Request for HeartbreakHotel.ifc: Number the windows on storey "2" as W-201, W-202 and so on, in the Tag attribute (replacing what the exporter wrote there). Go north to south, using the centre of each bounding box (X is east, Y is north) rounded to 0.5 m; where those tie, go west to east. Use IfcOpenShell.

First a look at what the model holds.

```python
import ifcopenshell
import ifcopenshell.util.element
import ifcopenshell.util.placement

model = ifcopenshell.open("HeartbreakHotel.ifc")
print(model.schema)
storey = next(s for s in model.by_type("IfcBuildingStorey") if s.Name == "2")
windows = [e for e in ifcopenshell.util.element.get_decomposition(storey) if e.is_a("IfcWindow")]
for e in sorted(windows, key=lambda e: e.id()):
    origin = ifcopenshell.util.placement.get_local_placement(e.ObjectPlacement)[:3, 3]
    print(e.id(), e.Tag, e.Name, origin.round(2) + 0.0, sep=" | ")
```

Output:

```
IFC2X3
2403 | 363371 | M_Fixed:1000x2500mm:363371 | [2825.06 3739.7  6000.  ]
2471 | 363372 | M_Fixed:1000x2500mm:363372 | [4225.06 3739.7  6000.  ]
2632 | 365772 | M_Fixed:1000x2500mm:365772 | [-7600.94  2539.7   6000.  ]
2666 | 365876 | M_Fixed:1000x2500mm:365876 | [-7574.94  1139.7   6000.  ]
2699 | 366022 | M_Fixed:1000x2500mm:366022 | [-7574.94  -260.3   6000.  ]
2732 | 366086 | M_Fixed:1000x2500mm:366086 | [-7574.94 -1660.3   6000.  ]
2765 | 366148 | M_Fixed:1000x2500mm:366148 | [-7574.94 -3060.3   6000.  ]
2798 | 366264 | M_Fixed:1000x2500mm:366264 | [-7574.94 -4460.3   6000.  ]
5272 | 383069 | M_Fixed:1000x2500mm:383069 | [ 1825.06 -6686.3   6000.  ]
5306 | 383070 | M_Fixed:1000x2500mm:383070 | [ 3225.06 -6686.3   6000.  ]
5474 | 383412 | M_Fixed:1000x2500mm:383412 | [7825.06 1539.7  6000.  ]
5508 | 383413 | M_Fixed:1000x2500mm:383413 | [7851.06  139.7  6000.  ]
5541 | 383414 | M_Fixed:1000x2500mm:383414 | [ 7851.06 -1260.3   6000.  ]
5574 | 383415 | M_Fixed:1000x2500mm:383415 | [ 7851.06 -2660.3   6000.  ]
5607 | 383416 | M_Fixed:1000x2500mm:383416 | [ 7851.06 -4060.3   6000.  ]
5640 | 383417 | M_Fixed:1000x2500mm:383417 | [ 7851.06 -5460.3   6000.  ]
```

```python
import ifcopenshell
import ifcopenshell.geom
import ifcopenshell.util.element
import ifcopenshell.util.shape

model = ifcopenshell.open("HeartbreakHotel.ifc")
settings = ifcopenshell.geom.settings()
settings.set("use-world-coords", True)


def centre(element):
    shape = ifcopenshell.geom.create_shape(settings, element)
    return ifcopenshell.util.shape.get_bbox_centroid(shape.geometry)


storey = next(s for s in model.by_type("IfcBuildingStorey") if s.Name == "2")
windows = [e for e in ifcopenshell.util.element.get_decomposition(storey) if e.is_a("IfcWindow")]

# Insertion points can sit at a corner or the storey origin, so sort by the geometry (in metres).
centres = {e: centre(e) for e in windows}
windows.sort(key=lambda e: (-round(centres[e][1] / 0.5), centres[e][0]))

for i, e in enumerate(windows, start=1):
    number = f"W-2{i:02d}"
    e.Tag = number
    print(e.id(), number)

model.write("HeartbreakHotel_edited.ifc")
```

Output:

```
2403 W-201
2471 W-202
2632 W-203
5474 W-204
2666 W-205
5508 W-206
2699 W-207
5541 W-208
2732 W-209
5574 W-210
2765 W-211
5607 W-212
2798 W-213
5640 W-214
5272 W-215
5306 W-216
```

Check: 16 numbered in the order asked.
